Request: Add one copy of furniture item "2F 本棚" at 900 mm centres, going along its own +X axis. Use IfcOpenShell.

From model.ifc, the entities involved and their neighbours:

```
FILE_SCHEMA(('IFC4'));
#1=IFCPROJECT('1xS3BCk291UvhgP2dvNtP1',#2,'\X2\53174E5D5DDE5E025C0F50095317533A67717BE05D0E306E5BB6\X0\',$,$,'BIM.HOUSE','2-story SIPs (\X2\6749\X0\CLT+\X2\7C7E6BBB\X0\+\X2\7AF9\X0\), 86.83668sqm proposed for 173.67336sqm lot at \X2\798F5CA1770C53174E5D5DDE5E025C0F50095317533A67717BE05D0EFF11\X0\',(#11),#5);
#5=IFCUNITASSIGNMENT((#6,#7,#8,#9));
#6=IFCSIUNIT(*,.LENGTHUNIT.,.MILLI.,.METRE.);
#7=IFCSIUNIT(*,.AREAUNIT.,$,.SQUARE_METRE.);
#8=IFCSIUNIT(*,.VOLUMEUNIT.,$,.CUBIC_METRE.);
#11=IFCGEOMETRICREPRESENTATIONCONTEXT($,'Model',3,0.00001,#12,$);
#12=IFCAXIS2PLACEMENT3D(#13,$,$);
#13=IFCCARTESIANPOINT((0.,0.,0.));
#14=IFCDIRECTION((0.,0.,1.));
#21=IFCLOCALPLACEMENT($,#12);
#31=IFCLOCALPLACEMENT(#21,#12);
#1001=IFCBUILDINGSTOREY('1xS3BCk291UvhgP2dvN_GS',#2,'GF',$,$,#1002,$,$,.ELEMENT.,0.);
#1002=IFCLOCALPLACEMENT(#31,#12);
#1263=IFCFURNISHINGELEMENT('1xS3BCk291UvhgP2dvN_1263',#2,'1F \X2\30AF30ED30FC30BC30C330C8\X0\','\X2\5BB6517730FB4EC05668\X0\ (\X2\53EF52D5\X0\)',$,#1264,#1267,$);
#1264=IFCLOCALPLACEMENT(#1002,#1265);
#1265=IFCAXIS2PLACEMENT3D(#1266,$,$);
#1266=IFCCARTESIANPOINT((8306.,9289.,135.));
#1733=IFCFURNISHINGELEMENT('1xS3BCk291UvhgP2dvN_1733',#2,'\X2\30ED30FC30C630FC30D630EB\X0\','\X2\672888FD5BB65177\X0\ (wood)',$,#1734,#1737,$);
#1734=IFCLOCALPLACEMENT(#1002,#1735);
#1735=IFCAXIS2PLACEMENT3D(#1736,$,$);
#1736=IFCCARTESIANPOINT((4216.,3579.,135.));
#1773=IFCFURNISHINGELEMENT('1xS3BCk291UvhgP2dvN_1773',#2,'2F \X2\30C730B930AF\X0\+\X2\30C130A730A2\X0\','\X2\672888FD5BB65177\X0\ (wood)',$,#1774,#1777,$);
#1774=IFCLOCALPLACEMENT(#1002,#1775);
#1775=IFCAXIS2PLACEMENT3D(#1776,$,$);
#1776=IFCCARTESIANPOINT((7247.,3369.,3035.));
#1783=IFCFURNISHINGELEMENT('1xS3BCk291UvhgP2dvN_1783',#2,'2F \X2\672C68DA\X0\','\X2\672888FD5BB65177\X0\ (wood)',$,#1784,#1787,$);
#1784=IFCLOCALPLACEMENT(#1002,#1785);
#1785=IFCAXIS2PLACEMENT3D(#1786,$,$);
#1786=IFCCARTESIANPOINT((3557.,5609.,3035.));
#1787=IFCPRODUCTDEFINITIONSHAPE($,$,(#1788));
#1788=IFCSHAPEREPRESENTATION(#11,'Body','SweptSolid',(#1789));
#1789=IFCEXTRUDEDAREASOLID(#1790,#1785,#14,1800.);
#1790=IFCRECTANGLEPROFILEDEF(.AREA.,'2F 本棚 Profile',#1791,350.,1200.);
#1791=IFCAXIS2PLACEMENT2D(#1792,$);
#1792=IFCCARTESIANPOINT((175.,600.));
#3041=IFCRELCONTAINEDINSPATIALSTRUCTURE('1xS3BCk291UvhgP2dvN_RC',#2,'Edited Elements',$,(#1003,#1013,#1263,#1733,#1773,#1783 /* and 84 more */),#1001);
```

```python
import ifcopenshell
import ifcopenshell.api.geometry
import ifcopenshell.api.root
import ifcopenshell.util.element
import ifcopenshell.util.placement
import ifcopenshell.util.unit

model = ifcopenshell.open("model.ifc")
unit_scale = ifcopenshell.util.unit.calculate_unit_scale(model)


def reuse_history(source, copy):
    """copy_class also copies each property set's owner history, people and application; keep the originals."""
    for rel in copy.IsDefinedBy:
        if rel.is_a("IfcRelDefinesByProperties") and (history := rel.RelatingPropertyDefinition.OwnerHistory):
            rel.RelatingPropertyDefinition.OwnerHistory = source.OwnerHistory
            ifcopenshell.util.element.remove_deep2(model, history)


source = model.by_guid("1xS3BCk291UvhgP2dvN_1783")
base = ifcopenshell.util.placement.get_local_placement(source.ObjectPlacement)
step = base[:3, 0] * 0.9 / unit_scale

for i in range(1, 2):
    copy = ifcopenshell.api.root.copy_class(model, product=source)
    copy.Representation = ifcopenshell.util.element.copy_deep(
        model, source.Representation, exclude=["IfcGeometricRepresentationContext", "IfcRepresentationMap"]
    )
    reuse_history(source, copy)
    matrix = base.copy()
    matrix[:3, 3] += i * step
    print("added at", matrix[:3, 3].round(3) + 0.0)
    ifcopenshell.api.geometry.edit_object_placement(model, product=copy, matrix=matrix, is_si=False)

model.write("model_rev.ifc")
```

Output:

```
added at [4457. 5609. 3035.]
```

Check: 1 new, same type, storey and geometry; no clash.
